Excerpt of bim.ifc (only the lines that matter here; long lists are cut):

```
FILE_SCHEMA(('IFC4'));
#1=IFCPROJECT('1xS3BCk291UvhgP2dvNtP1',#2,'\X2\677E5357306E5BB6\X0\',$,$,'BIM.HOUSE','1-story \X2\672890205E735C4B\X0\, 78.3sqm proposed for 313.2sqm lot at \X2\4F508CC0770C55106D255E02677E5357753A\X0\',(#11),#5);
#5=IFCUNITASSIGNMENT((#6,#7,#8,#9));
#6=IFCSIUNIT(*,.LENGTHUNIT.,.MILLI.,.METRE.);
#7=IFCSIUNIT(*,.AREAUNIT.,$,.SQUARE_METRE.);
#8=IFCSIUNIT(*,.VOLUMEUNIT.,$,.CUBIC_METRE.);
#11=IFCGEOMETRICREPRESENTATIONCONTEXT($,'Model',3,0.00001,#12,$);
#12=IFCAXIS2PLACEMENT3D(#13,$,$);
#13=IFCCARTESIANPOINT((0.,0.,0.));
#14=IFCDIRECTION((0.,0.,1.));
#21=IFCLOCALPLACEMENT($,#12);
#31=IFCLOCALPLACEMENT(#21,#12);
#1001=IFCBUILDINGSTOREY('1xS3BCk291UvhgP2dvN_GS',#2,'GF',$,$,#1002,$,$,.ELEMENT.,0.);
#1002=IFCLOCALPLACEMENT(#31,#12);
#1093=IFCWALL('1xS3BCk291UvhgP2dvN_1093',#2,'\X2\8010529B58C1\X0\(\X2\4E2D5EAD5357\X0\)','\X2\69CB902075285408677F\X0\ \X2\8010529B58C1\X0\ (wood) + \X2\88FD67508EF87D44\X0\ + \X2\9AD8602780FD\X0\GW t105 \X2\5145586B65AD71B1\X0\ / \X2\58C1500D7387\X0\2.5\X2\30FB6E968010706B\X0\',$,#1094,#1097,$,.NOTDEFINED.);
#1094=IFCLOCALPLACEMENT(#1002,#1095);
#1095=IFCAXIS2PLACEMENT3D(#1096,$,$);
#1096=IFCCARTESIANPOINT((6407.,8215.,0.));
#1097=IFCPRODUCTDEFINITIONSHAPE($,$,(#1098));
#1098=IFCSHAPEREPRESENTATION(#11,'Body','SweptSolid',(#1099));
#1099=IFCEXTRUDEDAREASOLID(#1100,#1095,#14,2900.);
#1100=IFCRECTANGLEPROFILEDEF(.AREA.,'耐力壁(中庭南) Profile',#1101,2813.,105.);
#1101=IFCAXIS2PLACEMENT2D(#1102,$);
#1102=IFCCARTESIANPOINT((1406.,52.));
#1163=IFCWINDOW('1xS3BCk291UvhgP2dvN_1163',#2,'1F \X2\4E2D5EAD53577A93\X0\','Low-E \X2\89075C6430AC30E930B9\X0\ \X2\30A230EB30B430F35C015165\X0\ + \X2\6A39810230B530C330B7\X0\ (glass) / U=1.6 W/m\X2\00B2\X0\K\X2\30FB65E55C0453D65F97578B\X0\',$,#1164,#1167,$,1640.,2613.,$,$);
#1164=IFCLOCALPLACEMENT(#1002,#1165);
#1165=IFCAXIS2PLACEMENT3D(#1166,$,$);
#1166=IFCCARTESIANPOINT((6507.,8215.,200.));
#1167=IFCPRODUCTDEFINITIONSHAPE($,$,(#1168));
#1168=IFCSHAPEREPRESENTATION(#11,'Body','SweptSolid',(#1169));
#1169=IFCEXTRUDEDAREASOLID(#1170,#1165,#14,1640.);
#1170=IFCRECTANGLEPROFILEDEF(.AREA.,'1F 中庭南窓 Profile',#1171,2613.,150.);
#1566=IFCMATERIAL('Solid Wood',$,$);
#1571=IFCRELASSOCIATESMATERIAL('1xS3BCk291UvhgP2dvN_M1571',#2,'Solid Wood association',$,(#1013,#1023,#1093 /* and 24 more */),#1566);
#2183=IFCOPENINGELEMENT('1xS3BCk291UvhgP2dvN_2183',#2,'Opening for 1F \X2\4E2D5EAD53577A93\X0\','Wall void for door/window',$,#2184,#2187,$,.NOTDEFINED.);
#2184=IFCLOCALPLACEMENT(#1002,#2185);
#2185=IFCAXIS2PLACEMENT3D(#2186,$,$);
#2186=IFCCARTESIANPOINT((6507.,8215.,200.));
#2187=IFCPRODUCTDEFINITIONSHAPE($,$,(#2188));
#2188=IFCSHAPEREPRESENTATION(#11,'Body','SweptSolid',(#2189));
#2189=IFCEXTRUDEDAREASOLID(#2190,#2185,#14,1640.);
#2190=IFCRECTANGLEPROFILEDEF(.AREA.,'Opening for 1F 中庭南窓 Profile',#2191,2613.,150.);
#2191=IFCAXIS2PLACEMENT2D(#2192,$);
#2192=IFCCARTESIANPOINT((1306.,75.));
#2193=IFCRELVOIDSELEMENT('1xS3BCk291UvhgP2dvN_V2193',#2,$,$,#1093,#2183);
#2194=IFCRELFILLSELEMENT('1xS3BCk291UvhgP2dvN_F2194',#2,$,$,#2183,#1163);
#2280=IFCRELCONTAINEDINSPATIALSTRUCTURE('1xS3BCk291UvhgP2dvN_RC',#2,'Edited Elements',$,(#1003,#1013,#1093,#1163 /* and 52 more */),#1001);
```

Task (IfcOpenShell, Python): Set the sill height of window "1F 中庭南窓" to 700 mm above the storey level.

```python
import numpy as np
import ifcopenshell
import ifcopenshell.api.geometry
import ifcopenshell.geom
import ifcopenshell.util.element
import ifcopenshell.util.placement
import ifcopenshell.util.shape
import ifcopenshell.util.unit

model = ifcopenshell.open("bim.ifc")
unit_scale = ifcopenshell.util.unit.calculate_unit_scale(model)

window = model.by_id(1163)
opening = window.FillsVoids[0].RelatingOpeningElement
storey = ifcopenshell.util.element.get_container(window, ifc_class="IfcBuildingStorey")
level = ifcopenshell.util.placement.get_local_placement(storey.ObjectPlacement)[2, 3]

# The opening's origin need not be at the sill, so measure its lowest point.
shape = ifcopenshell.geom.create_shape(ifcopenshell.geom.settings(), opening)
bottom = ifcopenshell.util.shape.get_shape_bottom_elevation(shape, shape.geometry) / unit_scale
dz = level + 0.7 / unit_scale - bottom

shift = np.array([0.0, 0.0, dz])
# The window is not placed relative to its opening, so move both.
for product in (opening, window):
    matrix = ifcopenshell.util.placement.get_local_placement(product.ObjectPlacement)
    matrix[:3, 3] += shift
    ifcopenshell.api.geometry.edit_object_placement(model, product=product, matrix=matrix, is_si=False)

print(f"moved by {dz * unit_scale:+.3f} m")

model.write("bim-out.ifc")
```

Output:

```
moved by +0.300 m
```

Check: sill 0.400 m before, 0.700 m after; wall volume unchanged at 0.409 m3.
